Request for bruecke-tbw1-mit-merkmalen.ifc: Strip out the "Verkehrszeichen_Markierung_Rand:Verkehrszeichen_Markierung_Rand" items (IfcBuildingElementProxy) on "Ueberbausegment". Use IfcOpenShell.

First a look at what the model holds.

```python
import ifcopenshell
import ifcopenshell.util.element

model = ifcopenshell.open("bruecke-tbw1-mit-merkmalen.ifc")
print(model.schema)
storey = next(s for s in model.by_type("IfcBuildingStorey") if s.Name == "Ueberbausegment")
proxies = [e for e in ifcopenshell.util.element.get_decomposition(storey) if e.is_a("IfcBuildingElementProxy")]
seen = {}
for e in proxies:
    element_type = ifcopenshell.util.element.get_type(e)
    name = element_type.Name if element_type not in (None, e) else None
    seen[name] = seen.get(name, 0) + 1
for name, count in sorted(seen.items(), key=str):
    print(count, "x", name)
```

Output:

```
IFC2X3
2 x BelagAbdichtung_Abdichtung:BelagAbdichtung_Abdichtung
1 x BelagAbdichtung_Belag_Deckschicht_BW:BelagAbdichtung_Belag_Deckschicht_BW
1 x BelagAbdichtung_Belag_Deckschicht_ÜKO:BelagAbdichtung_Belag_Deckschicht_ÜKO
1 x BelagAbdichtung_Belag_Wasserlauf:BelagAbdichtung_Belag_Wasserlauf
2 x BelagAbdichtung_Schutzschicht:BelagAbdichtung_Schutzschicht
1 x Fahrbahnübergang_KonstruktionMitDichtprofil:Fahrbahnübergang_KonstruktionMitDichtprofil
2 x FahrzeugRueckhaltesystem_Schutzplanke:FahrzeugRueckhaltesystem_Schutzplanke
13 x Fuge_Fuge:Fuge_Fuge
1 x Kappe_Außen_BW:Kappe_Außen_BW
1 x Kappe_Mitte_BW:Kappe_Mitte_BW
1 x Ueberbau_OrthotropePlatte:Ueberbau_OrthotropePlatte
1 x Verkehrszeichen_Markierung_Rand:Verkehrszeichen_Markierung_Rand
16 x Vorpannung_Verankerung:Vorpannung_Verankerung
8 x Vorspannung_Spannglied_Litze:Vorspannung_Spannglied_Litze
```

```python
import ifcopenshell
import ifcopenshell.api.root
import ifcopenshell.util.element

model = ifcopenshell.open("bruecke-tbw1-mit-merkmalen.ifc")

storey = next(s for s in model.by_type("IfcBuildingStorey") if s.Name == "Ueberbausegment")
proxies = [e for e in ifcopenshell.util.element.get_decomposition(storey) if e.is_a("IfcBuildingElementProxy")]
targets = [e for e in proxies if (t := ifcopenshell.util.element.get_type(e)) not in (None, e) and t.Name == "Verkehrszeichen_Markierung_Rand:Verkehrszeichen_Markierung_Rand"]

for e in targets:
    ifcopenshell.api.root.remove_product(model, product=e)
print(len(targets), "removed")

model.write("bruecke-tbw1-mit-merkmalen-out.ifc")
```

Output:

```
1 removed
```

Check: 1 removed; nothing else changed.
